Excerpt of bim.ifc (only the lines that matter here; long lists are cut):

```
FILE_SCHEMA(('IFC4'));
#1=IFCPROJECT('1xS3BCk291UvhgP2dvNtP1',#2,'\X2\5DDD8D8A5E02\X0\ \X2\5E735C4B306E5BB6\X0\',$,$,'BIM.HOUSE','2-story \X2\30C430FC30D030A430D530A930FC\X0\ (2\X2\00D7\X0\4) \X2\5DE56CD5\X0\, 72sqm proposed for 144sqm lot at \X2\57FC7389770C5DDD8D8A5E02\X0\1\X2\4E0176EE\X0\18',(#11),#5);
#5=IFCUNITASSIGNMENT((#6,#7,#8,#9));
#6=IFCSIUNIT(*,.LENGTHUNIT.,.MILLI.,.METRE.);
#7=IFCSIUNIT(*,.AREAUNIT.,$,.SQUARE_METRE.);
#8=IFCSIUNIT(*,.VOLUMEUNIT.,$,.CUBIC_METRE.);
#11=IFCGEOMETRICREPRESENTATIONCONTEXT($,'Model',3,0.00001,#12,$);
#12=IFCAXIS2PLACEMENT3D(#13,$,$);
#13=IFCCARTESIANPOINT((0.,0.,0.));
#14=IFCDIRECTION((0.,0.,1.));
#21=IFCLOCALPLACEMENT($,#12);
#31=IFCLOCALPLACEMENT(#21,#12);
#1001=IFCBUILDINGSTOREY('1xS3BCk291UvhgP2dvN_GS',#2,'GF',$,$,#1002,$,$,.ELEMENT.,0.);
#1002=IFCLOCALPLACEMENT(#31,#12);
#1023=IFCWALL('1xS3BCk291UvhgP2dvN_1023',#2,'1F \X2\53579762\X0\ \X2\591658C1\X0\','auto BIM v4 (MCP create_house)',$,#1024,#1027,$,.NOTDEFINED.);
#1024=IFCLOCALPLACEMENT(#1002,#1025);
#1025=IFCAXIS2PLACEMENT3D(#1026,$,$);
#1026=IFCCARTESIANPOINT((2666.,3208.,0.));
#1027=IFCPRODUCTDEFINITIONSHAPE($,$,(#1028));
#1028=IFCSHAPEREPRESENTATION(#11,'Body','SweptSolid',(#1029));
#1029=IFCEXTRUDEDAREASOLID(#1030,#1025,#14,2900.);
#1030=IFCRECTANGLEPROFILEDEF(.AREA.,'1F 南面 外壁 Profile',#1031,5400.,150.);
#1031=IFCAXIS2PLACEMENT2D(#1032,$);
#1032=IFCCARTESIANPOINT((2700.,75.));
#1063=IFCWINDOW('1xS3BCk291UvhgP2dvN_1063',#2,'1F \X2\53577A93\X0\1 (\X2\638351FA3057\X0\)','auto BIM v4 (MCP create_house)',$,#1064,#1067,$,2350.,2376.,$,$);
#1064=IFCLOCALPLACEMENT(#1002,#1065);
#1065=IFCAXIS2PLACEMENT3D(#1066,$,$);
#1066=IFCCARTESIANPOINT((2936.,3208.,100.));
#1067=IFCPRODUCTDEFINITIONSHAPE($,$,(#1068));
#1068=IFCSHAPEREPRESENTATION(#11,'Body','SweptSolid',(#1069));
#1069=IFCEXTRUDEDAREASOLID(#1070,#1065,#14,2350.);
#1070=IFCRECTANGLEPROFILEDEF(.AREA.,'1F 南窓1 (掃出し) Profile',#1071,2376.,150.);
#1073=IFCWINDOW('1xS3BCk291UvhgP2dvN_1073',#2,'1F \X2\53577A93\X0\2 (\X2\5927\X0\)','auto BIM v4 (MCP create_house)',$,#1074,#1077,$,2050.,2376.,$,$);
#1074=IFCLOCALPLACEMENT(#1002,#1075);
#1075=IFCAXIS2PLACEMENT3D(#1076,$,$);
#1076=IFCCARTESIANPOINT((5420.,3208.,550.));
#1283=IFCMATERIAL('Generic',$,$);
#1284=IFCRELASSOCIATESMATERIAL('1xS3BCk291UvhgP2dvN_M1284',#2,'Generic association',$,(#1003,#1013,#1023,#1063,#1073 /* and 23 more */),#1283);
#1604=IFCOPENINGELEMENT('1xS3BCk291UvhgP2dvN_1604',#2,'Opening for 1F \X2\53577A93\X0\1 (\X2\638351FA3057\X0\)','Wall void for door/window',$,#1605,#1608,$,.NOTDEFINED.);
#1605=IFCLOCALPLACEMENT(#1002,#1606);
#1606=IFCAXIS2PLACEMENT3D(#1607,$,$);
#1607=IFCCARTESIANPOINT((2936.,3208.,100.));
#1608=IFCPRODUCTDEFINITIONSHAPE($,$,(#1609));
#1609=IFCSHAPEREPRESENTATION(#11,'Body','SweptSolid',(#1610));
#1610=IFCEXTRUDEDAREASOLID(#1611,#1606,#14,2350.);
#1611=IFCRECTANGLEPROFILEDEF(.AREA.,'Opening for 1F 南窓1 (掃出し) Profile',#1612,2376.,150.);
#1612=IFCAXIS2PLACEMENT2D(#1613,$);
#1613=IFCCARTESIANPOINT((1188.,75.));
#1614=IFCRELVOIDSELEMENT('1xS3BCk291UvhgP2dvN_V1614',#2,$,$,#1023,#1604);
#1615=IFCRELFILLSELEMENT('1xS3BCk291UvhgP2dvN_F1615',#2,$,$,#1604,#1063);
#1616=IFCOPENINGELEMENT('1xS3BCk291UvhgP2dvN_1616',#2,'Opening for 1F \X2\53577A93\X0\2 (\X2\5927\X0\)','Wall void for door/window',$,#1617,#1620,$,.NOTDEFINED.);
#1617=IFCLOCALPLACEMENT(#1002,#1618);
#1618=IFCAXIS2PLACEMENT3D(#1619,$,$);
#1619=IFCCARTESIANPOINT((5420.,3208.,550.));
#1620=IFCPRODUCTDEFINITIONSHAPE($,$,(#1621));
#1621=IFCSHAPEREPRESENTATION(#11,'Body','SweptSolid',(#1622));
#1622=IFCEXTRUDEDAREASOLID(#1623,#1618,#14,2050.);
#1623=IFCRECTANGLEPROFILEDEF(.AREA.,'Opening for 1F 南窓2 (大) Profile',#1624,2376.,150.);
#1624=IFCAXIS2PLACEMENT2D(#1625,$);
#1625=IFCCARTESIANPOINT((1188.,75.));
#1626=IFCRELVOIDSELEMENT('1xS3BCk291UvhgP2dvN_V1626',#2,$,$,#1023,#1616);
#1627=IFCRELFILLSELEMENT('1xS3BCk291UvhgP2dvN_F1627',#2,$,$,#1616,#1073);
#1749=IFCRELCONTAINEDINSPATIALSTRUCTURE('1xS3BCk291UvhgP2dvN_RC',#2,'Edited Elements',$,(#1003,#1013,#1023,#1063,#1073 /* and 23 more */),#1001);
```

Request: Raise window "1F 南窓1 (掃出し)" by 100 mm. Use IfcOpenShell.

```python
import numpy as np
import ifcopenshell
import ifcopenshell.api.geometry
import ifcopenshell.util.placement
import ifcopenshell.util.unit

model = ifcopenshell.open("bim.ifc")
unit_scale = ifcopenshell.util.unit.calculate_unit_scale(model)

window = model.by_guid("1xS3BCk291UvhgP2dvN_1063")
opening = window.FillsVoids[0].RelatingOpeningElement
dz = 0.1 / unit_scale

shift = np.array([0.0, 0.0, dz])
# The window is not placed relative to its opening, so move both.
for product in (opening, window):
    matrix = ifcopenshell.util.placement.get_local_placement(product.ObjectPlacement)
    matrix[:3, 3] += shift
    ifcopenshell.api.geometry.edit_object_placement(model, product=product, matrix=matrix, is_si=False)

print(f"moved by {dz * unit_scale:+.3f} m")

model.write("bim_v2.ifc")
```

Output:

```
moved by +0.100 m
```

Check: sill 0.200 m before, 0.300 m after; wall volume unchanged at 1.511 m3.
